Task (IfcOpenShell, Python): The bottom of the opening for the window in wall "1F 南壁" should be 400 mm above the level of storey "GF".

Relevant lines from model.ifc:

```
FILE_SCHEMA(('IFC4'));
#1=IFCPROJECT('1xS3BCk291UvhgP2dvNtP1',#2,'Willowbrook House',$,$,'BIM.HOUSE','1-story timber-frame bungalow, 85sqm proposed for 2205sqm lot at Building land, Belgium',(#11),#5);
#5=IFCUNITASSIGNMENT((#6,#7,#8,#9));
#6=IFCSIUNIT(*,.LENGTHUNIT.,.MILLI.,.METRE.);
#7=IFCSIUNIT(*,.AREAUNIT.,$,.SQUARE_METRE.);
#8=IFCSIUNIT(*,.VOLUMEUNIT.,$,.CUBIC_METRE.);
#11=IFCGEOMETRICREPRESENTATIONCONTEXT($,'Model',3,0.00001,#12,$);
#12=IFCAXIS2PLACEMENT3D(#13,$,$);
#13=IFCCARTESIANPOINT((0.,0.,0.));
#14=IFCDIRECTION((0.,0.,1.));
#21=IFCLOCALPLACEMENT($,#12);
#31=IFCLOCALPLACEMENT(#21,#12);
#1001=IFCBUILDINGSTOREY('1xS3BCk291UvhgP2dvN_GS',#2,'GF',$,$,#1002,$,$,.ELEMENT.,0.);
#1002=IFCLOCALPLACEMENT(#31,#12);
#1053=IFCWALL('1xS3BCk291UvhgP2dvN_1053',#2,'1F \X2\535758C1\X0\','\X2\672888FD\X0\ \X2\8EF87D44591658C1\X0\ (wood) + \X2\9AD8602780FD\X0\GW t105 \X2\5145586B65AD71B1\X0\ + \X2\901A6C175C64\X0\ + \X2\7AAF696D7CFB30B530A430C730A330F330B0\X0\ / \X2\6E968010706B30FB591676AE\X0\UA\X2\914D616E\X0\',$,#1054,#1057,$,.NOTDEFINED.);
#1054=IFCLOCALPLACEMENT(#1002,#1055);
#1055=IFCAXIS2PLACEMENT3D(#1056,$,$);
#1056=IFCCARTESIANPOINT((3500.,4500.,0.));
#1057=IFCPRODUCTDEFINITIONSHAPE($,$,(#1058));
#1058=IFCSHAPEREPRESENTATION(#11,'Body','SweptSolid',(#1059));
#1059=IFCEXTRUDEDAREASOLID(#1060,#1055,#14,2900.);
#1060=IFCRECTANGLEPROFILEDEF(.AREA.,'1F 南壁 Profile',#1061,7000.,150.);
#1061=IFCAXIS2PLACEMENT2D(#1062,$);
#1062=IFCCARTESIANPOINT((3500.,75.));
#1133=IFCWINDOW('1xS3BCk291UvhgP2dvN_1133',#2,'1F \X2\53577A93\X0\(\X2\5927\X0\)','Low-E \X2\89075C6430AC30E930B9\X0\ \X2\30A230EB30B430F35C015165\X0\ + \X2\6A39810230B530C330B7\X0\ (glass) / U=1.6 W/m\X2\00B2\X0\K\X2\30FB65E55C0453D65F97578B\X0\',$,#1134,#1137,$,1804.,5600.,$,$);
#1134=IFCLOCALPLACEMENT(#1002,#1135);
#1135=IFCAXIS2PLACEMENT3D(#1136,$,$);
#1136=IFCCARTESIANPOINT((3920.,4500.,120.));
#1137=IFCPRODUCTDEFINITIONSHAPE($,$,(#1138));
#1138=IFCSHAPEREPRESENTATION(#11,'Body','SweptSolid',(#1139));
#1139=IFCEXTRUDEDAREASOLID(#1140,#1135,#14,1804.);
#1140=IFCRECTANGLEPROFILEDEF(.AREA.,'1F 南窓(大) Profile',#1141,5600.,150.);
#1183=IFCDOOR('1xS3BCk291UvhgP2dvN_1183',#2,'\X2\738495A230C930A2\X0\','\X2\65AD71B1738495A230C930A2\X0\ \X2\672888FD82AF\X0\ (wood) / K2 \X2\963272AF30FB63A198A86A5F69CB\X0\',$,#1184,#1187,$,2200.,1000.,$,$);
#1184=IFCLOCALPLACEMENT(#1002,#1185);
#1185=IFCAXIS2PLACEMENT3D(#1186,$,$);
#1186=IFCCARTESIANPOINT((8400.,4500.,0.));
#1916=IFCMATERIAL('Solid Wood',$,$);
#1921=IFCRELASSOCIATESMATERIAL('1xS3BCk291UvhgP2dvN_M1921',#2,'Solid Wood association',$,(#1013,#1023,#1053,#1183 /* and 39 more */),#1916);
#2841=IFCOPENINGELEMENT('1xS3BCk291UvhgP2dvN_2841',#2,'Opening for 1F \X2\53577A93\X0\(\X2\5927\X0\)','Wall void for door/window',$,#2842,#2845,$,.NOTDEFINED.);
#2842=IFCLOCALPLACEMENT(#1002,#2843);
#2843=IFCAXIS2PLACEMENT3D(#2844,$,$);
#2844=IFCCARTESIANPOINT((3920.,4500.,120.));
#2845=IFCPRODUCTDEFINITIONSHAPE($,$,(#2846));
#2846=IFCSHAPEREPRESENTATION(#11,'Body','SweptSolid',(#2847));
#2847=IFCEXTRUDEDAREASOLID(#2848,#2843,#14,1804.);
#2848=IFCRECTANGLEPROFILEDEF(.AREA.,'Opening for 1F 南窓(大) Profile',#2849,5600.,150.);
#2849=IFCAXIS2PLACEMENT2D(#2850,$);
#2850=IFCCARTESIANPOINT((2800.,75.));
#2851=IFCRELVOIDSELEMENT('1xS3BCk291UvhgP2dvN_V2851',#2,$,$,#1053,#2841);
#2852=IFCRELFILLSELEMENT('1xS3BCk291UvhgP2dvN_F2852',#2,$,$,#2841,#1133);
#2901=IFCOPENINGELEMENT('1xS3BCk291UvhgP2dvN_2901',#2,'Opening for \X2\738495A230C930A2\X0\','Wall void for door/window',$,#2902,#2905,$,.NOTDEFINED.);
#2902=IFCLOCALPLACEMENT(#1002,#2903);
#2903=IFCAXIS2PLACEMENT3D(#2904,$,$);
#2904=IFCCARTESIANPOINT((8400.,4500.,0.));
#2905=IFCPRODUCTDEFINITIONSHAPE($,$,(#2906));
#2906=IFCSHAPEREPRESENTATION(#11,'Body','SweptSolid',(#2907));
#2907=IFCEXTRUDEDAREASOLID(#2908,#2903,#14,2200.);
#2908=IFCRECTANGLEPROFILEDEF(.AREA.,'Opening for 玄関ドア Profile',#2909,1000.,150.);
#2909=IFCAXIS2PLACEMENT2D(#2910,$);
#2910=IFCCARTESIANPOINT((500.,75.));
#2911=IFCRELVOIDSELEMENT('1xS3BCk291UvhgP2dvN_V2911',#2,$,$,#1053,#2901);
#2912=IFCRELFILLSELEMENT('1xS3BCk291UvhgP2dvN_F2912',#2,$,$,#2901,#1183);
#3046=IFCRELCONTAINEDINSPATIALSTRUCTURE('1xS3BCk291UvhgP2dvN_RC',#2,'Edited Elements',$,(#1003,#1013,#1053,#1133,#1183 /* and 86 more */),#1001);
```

```python
import numpy as np
import ifcopenshell
import ifcopenshell.api.geometry
import ifcopenshell.geom
import ifcopenshell.util.element
import ifcopenshell.util.placement
import ifcopenshell.util.shape
import ifcopenshell.util.unit

model = ifcopenshell.open("model.ifc")
unit_scale = ifcopenshell.util.unit.calculate_unit_scale(model)

window = model.by_id(1133)
opening = window.FillsVoids[0].RelatingOpeningElement
storey = ifcopenshell.util.element.get_container(window, ifc_class="IfcBuildingStorey")
level = ifcopenshell.util.placement.get_local_placement(storey.ObjectPlacement)[2, 3]

# The opening's origin need not be at the sill, so measure its lowest point.
shape = ifcopenshell.geom.create_shape(ifcopenshell.geom.settings(), opening)
bottom = ifcopenshell.util.shape.get_shape_bottom_elevation(shape, shape.geometry) / unit_scale
dz = level + 400.0 - bottom

shift = np.array([0.0, 0.0, dz])
# The window is not placed relative to its opening, so move both.
for product in (opening, window):
    matrix = ifcopenshell.util.placement.get_local_placement(product.ObjectPlacement)
    matrix[:3, 3] += shift
    ifcopenshell.api.geometry.edit_object_placement(model, product=product, matrix=matrix, is_si=False)

print(f"moved by {dz * unit_scale:+.3f} m")

model.write("model_v2.ifc")
```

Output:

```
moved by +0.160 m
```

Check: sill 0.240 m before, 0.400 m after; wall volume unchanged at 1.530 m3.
